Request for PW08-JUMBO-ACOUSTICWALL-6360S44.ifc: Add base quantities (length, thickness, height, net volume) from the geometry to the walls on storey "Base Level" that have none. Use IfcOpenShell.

First a look at what the model holds.

```python
import ifcopenshell
import ifcopenshell.util.element
import ifcopenshell.util.unit

model = ifcopenshell.open("PW08-JUMBO-ACOUSTICWALL-6360S44.ifc")
print(model.schema)
for unit_type in ("LENGTHUNIT", "AREAUNIT", "VOLUMEUNIT"):
    print(unit_type, ifcopenshell.util.unit.calculate_unit_scale(model, unit_type))
storey = next(s for s in model.by_type("IfcBuildingStorey") if s.Name == "Base Level")
walls = [e for e in ifcopenshell.util.element.get_decomposition(storey) if e.is_a("IfcWall")]
for e in sorted(walls, key=lambda e: e.id()):
    print(e.id(), e.is_a(), e.Name, list(ifcopenshell.util.element.get_psets(e, qtos_only=True)), sep=" | ")
```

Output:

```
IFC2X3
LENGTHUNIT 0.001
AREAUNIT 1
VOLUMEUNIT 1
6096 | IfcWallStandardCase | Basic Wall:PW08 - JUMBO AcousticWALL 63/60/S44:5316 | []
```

```python
import ifcopenshell
import ifcopenshell.api.pset
import ifcopenshell.geom
import ifcopenshell.util.element
import ifcopenshell.util.shape
import ifcopenshell.util.unit

model = ifcopenshell.open("PW08-JUMBO-ACOUSTICWALL-6360S44.ifc")
unit_scale = ifcopenshell.util.unit.calculate_unit_scale(model)
volume_scale = ifcopenshell.util.unit.calculate_unit_scale(model, "VOLUMEUNIT")
settings = ifcopenshell.geom.settings()

storey = next(s for s in model.by_type("IfcBuildingStorey") if s.Name == "Base Level")
walls = [e for e in ifcopenshell.util.element.get_decomposition(storey) if e.is_a("IfcWall")]

for e in sorted(walls, key=lambda e: e.id()):
    if ifcopenshell.util.element.get_psets(e, qtos_only=True, should_inherit=False):
        continue
    # Geometry comes back in metres, in the element's own axes.
    shape = ifcopenshell.geom.create_shape(settings, e)
    values = {
        "Length": ifcopenshell.util.shape.get_x(shape.geometry) / unit_scale,
        "Width": ifcopenshell.util.shape.get_y(shape.geometry) / unit_scale,
        "Height": ifcopenshell.util.shape.get_z(shape.geometry) / unit_scale,
        "NetVolume": ifcopenshell.util.shape.get_volume(shape.geometry) / volume_scale,
    }
    qto = ifcopenshell.api.pset.add_qto(model, product=e, name="BaseQuantities")
    ifcopenshell.api.pset.edit_qto(model, qto=qto, properties=values)
    print(e.id(), {k: round(v, 3) for k, v in values.items()})

model.write("PW08-JUMBO-ACOUSTICWALL-6360S44_v2.ifc")
```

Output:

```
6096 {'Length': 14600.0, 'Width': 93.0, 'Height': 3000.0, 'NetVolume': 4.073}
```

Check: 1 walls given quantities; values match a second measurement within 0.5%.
